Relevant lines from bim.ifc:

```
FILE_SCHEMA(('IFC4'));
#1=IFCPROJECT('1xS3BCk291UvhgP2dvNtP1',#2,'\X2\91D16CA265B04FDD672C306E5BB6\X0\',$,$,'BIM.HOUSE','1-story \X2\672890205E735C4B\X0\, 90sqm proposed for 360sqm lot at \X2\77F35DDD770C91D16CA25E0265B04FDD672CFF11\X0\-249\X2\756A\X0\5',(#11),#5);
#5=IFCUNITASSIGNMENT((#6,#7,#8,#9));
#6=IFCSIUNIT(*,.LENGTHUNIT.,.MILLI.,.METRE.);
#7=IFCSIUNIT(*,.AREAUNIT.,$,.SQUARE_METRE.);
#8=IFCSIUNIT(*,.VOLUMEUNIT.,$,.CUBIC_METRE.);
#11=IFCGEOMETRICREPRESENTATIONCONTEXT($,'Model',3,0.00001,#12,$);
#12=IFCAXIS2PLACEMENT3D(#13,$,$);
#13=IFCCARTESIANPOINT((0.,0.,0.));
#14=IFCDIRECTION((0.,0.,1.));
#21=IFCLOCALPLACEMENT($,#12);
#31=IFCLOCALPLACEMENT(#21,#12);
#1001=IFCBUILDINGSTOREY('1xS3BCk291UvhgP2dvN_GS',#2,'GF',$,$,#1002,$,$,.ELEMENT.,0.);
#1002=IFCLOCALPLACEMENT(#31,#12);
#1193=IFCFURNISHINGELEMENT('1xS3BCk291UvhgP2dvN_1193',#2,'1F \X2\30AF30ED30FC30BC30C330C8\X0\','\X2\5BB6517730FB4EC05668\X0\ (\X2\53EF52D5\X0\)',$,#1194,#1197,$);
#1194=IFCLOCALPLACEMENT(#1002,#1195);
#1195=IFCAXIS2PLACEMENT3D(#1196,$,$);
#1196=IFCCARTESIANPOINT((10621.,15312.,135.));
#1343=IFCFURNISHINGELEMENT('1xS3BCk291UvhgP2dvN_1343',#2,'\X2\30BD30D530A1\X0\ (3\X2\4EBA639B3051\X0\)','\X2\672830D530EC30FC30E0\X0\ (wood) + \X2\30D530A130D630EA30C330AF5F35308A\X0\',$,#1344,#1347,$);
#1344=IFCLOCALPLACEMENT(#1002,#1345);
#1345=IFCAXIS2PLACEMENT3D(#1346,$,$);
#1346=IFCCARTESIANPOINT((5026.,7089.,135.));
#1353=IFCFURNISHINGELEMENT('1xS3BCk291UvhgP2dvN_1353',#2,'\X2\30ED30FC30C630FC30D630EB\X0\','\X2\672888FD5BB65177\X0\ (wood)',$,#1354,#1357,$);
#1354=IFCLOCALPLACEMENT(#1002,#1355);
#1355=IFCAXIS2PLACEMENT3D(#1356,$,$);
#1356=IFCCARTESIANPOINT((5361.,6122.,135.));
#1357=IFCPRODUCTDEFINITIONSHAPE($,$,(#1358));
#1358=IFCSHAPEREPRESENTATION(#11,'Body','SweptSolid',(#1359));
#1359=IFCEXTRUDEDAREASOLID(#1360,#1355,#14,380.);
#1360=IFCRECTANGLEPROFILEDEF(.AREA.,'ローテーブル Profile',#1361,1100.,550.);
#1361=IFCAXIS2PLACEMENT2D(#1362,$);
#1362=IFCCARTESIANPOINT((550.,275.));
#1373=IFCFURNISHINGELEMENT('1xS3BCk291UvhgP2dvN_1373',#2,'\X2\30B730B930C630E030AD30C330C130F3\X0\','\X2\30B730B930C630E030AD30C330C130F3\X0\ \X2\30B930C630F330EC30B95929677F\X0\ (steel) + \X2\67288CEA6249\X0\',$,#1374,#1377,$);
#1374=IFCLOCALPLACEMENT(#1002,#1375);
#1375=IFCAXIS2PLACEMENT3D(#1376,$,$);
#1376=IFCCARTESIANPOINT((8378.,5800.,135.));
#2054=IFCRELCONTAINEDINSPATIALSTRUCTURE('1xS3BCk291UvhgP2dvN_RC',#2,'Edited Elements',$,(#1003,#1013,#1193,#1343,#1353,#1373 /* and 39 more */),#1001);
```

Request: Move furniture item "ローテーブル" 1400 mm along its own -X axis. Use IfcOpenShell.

```python
import ifcopenshell
import ifcopenshell.api.geometry
import ifcopenshell.util.placement

model = ifcopenshell.open("bim.ifc")

item = model.by_guid("1xS3BCk291UvhgP2dvN_1353")
matrix = ifcopenshell.util.placement.get_local_placement(item.ObjectPlacement)
matrix[:3, 3] -= matrix[:3, 0] * 1400.0
ifcopenshell.api.geometry.edit_object_placement(model, product=item, matrix=matrix, is_si=False)

print(ifcopenshell.util.placement.get_local_placement(item.ObjectPlacement).round(3) + 0.0)

model.write("bim_v2.ifc")
```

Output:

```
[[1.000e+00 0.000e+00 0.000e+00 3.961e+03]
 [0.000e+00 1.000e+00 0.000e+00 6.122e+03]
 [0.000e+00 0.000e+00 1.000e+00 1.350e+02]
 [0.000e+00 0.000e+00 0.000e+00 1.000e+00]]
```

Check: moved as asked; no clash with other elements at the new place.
